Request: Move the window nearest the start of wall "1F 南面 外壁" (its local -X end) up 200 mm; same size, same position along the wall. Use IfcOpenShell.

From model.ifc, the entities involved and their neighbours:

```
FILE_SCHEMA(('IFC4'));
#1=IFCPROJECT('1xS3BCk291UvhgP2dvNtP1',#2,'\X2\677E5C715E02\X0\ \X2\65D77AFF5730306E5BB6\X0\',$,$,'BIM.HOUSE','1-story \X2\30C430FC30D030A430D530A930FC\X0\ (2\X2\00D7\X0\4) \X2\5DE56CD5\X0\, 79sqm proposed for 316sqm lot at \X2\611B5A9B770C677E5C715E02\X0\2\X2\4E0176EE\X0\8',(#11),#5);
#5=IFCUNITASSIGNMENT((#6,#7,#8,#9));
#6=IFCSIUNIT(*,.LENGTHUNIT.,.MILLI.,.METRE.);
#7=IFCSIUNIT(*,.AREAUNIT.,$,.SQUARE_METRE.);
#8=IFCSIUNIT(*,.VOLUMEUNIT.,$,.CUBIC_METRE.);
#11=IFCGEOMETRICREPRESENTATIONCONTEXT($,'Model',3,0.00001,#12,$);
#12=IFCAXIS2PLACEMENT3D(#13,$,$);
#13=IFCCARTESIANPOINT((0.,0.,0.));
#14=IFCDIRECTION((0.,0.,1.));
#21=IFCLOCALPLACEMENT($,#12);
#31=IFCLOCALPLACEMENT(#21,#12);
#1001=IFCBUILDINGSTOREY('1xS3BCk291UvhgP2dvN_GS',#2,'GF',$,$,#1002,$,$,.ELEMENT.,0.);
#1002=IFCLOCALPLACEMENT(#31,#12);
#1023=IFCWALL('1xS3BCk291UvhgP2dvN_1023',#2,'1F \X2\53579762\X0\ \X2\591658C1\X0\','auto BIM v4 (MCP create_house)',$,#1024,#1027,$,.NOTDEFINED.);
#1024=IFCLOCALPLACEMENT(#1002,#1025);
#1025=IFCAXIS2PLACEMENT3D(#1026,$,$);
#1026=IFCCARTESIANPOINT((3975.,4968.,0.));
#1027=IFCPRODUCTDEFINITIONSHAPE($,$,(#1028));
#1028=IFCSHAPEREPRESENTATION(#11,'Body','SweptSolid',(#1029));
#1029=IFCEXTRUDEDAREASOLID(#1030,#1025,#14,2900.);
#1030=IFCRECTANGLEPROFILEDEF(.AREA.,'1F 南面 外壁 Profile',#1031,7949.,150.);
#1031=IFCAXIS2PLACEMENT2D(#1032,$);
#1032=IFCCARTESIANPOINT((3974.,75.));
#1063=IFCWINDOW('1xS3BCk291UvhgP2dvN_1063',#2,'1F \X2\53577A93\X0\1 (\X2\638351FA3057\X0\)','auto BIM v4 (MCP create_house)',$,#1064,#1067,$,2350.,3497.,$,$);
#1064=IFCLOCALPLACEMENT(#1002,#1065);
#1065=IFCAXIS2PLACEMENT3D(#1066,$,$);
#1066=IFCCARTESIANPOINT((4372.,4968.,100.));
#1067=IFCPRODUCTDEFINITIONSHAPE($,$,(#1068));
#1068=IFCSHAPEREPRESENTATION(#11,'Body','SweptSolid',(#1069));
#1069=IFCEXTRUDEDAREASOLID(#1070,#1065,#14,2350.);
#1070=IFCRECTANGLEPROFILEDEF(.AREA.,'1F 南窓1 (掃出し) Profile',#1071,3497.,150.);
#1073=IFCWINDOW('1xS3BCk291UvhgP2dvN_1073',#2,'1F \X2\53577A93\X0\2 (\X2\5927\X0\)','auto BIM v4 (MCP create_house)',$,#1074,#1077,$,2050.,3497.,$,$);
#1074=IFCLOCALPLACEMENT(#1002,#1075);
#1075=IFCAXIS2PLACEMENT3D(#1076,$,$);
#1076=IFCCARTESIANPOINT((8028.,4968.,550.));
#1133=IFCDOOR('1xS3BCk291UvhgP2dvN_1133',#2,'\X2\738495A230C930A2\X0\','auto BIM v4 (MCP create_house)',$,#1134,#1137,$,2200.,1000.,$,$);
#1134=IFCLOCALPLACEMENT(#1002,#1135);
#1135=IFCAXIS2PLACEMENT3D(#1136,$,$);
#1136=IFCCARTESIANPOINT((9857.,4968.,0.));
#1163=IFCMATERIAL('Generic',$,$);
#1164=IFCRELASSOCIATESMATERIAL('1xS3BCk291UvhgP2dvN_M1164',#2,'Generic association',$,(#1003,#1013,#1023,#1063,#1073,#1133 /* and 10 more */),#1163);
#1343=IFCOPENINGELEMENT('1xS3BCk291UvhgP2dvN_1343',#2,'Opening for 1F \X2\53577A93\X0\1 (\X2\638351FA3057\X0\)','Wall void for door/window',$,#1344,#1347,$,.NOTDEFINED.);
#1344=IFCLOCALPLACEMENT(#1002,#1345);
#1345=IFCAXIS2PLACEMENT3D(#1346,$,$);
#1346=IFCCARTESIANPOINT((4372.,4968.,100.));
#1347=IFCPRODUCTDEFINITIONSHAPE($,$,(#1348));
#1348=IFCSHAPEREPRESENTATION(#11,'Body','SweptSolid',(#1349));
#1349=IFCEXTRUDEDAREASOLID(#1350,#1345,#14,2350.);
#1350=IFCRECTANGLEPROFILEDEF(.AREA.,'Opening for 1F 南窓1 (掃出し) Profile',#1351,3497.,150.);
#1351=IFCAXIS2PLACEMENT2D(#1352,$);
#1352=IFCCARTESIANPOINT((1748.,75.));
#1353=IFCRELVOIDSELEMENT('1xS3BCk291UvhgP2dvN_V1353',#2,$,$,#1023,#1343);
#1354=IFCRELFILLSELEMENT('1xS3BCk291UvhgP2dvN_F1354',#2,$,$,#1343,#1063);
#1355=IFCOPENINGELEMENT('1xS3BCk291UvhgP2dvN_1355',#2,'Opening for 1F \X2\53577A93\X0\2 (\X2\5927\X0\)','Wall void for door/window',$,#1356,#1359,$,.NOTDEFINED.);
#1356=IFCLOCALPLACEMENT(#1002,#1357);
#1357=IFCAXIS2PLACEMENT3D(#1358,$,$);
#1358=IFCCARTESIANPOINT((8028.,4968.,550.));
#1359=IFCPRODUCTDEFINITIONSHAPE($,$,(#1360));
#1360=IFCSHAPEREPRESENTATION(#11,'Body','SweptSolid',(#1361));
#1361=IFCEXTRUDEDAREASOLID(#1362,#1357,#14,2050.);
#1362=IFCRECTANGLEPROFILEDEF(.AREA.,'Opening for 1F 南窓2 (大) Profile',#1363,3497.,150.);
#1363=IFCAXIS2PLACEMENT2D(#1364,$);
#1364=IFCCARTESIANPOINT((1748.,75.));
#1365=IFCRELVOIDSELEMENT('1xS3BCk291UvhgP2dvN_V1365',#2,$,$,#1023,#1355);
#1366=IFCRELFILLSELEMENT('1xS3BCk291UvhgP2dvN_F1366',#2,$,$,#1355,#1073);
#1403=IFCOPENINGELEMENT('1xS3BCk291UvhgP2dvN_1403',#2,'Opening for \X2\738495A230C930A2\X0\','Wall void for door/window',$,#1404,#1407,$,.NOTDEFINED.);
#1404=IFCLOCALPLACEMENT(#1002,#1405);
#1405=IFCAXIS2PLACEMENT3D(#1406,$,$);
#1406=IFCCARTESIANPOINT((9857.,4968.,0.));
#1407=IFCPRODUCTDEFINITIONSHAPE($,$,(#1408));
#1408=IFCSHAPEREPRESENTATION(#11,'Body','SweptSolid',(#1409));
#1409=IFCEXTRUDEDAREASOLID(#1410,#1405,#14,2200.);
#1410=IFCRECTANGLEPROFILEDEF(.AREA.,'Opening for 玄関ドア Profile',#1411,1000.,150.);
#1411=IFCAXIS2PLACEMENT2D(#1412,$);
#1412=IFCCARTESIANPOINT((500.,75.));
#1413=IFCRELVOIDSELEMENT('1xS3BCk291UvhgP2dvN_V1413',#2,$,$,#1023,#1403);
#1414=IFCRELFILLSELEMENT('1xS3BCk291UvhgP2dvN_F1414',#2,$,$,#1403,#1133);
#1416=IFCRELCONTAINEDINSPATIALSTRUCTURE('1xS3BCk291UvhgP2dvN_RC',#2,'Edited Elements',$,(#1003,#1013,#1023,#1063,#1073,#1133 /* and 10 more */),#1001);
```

```python
import numpy as np
import ifcopenshell
import ifcopenshell.api.geometry
import ifcopenshell.util.placement
import ifcopenshell.util.unit

model = ifcopenshell.open("model.ifc")
unit_scale = ifcopenshell.util.unit.calculate_unit_scale(model)

window = model.by_guid("1xS3BCk291UvhgP2dvN_1063")
opening = window.FillsVoids[0].RelatingOpeningElement
dz = 200.0

shift = np.array([0.0, 0.0, dz])
# The window is not placed relative to its opening, so move both.
for product in (opening, window):
    matrix = ifcopenshell.util.placement.get_local_placement(product.ObjectPlacement)
    matrix[:3, 3] += shift
    ifcopenshell.api.geometry.edit_object_placement(model, product=product, matrix=matrix, is_si=False)

print(f"moved by {dz * unit_scale:+.3f} m")

model.write("model_updated.ifc")
```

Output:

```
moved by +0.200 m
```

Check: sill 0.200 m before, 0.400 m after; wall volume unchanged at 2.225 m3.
